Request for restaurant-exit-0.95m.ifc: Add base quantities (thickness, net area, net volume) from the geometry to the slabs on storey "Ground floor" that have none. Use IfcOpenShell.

First a look at what the model holds.

```python
import ifcopenshell
import ifcopenshell.util.element
import ifcopenshell.util.unit

model = ifcopenshell.open("restaurant-exit-0.95m.ifc")
print(model.schema)
for unit_type in ("LENGTHUNIT", "AREAUNIT", "VOLUMEUNIT"):
    print(unit_type, ifcopenshell.util.unit.calculate_unit_scale(model, unit_type))
storey = next(s for s in model.by_type("IfcBuildingStorey") if s.Name == "Ground floor")
slabs = [e for e in ifcopenshell.util.element.get_decomposition(storey) if e.is_a("IfcSlab")]
for e in sorted(slabs, key=lambda e: e.id()):
    print(e.id(), e.is_a(), e.Name, list(ifcopenshell.util.element.get_psets(e, qtos_only=True)), sep=" | ")
```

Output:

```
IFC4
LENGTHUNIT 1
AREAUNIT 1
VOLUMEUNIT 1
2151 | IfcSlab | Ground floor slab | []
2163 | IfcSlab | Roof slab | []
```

```python
import ifcopenshell
import ifcopenshell.api.pset
import ifcopenshell.geom
import ifcopenshell.util.element
import ifcopenshell.util.shape
import ifcopenshell.util.unit

model = ifcopenshell.open("restaurant-exit-0.95m.ifc")
unit_scale = ifcopenshell.util.unit.calculate_unit_scale(model)
area_scale = ifcopenshell.util.unit.calculate_unit_scale(model, "AREAUNIT")
volume_scale = ifcopenshell.util.unit.calculate_unit_scale(model, "VOLUMEUNIT")
settings = ifcopenshell.geom.settings()

storey = next(s for s in model.by_type("IfcBuildingStorey") if s.Name == "Ground floor")
slabs = [e for e in ifcopenshell.util.element.get_decomposition(storey) if e.is_a("IfcSlab")]

for e in sorted(slabs, key=lambda e: e.id()):
    if ifcopenshell.util.element.get_psets(e, qtos_only=True, should_inherit=False):
        continue
    # Geometry comes back in metres, in the element's own axes.
    shape = ifcopenshell.geom.create_shape(settings, e)
    values = {
        "Width": ifcopenshell.util.shape.get_z(shape.geometry) / unit_scale,
        "NetArea": ifcopenshell.util.shape.get_footprint_area(shape.geometry) / area_scale,
        "NetVolume": ifcopenshell.util.shape.get_volume(shape.geometry) / volume_scale,
    }
    qto = ifcopenshell.api.pset.add_qto(model, product=e, name="Qto_SlabBaseQuantities")
    ifcopenshell.api.pset.edit_qto(model, qto=qto, properties=values)
    print(e.id(), {k: round(v, 3) for k, v in values.items()})

model.write("restaurant-exit-0.95m_rev.ifc")
```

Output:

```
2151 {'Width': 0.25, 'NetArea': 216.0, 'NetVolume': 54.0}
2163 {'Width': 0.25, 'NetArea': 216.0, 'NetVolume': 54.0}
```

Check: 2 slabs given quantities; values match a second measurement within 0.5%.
